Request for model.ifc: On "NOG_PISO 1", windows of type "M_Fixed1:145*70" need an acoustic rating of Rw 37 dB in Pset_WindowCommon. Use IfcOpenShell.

First a look at what the model holds.

```python
import ifcopenshell
import ifcopenshell.util.element

model = ifcopenshell.open("model.ifc")
print(model.schema)
storey = next(s for s in model.by_type("IfcBuildingStorey") if s.Name == "NOG_PISO 1")
windows = [e for e in ifcopenshell.util.element.get_decomposition(storey) if e.is_a("IfcWindow")]
seen = {}
for e in windows:
    element_type = ifcopenshell.util.element.get_type(e)
    key = (element_type.Name if element_type != e and element_type else None, ifcopenshell.util.element.get_pset(e, "Pset_WindowCommon", "AcousticRating"))
    seen[key] = seen.get(key, 0) + 1
for (name, value), count in sorted(seen.items(), key=str):
    print(count, "x", name, "|", value)
```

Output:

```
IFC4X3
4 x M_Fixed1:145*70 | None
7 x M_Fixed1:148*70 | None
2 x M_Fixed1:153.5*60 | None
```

```python
import ifcopenshell
import ifcopenshell.api.pset
import ifcopenshell.util.element

model = ifcopenshell.open("model.ifc")

storey = next(s for s in model.by_type("IfcBuildingStorey") if s.Name == "NOG_PISO 1")
windows = [e for e in ifcopenshell.util.element.get_decomposition(storey) if e.is_a("IfcWindow")]

count = 0
for e in windows:
    element_type = ifcopenshell.util.element.get_type(e)
    if element_type in (None, e) or element_type.Name != "M_Fixed1:145*70":
        continue
    # add_pset returns the element's existing set when there is one.
    pset = ifcopenshell.api.pset.add_pset(model, product=e, name="Pset_WindowCommon")
    ifcopenshell.api.pset.edit_pset(model, pset=pset, properties={"AcousticRating": "Rw 37 dB"})
    count += 1

print(count, "windows updated")

model.write("model_updated.ifc")
```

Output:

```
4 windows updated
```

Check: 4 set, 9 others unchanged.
